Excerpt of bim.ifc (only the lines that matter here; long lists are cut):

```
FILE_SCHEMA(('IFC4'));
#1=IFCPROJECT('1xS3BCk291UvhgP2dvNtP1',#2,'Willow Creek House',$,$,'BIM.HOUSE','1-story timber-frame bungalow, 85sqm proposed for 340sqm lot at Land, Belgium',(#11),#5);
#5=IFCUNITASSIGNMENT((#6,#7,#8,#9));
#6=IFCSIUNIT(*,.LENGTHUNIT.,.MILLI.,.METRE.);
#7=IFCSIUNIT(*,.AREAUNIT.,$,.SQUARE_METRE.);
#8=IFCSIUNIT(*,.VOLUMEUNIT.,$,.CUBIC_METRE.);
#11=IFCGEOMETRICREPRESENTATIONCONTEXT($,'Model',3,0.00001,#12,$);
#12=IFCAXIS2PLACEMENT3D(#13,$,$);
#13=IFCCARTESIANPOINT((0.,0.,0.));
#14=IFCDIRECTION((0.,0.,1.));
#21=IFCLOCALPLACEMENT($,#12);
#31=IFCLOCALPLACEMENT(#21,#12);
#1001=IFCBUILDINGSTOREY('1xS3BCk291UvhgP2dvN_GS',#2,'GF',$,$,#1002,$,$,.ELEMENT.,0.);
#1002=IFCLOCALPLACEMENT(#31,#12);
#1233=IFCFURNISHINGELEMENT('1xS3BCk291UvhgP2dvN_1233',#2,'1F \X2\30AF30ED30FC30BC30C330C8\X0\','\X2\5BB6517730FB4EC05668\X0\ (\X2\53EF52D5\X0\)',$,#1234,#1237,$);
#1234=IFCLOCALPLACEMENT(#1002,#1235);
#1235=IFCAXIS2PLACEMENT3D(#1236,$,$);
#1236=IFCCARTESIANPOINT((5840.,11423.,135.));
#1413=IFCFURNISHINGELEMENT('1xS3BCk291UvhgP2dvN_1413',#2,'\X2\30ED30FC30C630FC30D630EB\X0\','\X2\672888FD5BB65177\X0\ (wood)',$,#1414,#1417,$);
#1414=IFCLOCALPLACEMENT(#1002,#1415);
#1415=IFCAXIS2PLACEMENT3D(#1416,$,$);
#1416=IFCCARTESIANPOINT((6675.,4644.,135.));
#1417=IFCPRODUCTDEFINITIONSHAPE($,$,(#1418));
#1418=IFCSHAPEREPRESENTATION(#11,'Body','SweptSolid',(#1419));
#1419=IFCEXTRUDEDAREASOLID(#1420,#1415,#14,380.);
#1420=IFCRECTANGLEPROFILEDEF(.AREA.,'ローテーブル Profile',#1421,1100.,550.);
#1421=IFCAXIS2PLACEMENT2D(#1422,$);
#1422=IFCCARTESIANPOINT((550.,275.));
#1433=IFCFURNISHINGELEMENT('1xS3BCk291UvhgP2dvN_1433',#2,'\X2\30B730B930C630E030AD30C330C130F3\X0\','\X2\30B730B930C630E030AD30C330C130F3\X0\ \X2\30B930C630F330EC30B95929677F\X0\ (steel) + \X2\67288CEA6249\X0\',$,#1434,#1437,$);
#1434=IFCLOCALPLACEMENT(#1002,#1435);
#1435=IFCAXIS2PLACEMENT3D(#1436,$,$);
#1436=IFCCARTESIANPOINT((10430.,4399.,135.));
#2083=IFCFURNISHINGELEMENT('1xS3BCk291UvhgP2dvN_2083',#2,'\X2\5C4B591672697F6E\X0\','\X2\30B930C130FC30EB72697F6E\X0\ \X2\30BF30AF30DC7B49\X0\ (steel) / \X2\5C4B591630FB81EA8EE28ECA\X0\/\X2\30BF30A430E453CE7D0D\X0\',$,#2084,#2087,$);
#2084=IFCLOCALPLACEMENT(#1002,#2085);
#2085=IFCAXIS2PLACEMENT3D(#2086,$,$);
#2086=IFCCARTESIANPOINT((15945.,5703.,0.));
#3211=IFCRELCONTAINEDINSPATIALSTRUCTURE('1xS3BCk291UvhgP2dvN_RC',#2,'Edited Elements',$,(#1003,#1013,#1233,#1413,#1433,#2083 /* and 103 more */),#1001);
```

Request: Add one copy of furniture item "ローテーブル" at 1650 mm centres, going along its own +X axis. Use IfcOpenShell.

```python
import ifcopenshell
import ifcopenshell.api.geometry
import ifcopenshell.api.root
import ifcopenshell.util.element
import ifcopenshell.util.placement

model = ifcopenshell.open("bim.ifc")


def reuse_history(source, copy):
    """copy_class also copies each property set's owner history, people and application; keep the originals."""
    for rel in copy.IsDefinedBy:
        if rel.is_a("IfcRelDefinesByProperties") and (history := rel.RelatingPropertyDefinition.OwnerHistory):
            rel.RelatingPropertyDefinition.OwnerHistory = source.OwnerHistory
            ifcopenshell.util.element.remove_deep2(model, history)


source = model.by_guid("1xS3BCk291UvhgP2dvN_1413")
base = ifcopenshell.util.placement.get_local_placement(source.ObjectPlacement)
step = base[:3, 0] * 1650.0

for i in range(1, 2):
    copy = ifcopenshell.api.root.copy_class(model, product=source)
    copy.Representation = ifcopenshell.util.element.copy_deep(
        model, source.Representation, exclude=["IfcGeometricRepresentationContext", "IfcRepresentationMap"]
    )
    reuse_history(source, copy)
    matrix = base.copy()
    matrix[:3, 3] += i * step
    print("added at", matrix[:3, 3].round(3) + 0.0)
    ifcopenshell.api.geometry.edit_object_placement(model, product=copy, matrix=matrix, is_si=False)

model.write("bim_rev.ifc")
```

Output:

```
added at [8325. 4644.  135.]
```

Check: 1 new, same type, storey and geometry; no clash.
